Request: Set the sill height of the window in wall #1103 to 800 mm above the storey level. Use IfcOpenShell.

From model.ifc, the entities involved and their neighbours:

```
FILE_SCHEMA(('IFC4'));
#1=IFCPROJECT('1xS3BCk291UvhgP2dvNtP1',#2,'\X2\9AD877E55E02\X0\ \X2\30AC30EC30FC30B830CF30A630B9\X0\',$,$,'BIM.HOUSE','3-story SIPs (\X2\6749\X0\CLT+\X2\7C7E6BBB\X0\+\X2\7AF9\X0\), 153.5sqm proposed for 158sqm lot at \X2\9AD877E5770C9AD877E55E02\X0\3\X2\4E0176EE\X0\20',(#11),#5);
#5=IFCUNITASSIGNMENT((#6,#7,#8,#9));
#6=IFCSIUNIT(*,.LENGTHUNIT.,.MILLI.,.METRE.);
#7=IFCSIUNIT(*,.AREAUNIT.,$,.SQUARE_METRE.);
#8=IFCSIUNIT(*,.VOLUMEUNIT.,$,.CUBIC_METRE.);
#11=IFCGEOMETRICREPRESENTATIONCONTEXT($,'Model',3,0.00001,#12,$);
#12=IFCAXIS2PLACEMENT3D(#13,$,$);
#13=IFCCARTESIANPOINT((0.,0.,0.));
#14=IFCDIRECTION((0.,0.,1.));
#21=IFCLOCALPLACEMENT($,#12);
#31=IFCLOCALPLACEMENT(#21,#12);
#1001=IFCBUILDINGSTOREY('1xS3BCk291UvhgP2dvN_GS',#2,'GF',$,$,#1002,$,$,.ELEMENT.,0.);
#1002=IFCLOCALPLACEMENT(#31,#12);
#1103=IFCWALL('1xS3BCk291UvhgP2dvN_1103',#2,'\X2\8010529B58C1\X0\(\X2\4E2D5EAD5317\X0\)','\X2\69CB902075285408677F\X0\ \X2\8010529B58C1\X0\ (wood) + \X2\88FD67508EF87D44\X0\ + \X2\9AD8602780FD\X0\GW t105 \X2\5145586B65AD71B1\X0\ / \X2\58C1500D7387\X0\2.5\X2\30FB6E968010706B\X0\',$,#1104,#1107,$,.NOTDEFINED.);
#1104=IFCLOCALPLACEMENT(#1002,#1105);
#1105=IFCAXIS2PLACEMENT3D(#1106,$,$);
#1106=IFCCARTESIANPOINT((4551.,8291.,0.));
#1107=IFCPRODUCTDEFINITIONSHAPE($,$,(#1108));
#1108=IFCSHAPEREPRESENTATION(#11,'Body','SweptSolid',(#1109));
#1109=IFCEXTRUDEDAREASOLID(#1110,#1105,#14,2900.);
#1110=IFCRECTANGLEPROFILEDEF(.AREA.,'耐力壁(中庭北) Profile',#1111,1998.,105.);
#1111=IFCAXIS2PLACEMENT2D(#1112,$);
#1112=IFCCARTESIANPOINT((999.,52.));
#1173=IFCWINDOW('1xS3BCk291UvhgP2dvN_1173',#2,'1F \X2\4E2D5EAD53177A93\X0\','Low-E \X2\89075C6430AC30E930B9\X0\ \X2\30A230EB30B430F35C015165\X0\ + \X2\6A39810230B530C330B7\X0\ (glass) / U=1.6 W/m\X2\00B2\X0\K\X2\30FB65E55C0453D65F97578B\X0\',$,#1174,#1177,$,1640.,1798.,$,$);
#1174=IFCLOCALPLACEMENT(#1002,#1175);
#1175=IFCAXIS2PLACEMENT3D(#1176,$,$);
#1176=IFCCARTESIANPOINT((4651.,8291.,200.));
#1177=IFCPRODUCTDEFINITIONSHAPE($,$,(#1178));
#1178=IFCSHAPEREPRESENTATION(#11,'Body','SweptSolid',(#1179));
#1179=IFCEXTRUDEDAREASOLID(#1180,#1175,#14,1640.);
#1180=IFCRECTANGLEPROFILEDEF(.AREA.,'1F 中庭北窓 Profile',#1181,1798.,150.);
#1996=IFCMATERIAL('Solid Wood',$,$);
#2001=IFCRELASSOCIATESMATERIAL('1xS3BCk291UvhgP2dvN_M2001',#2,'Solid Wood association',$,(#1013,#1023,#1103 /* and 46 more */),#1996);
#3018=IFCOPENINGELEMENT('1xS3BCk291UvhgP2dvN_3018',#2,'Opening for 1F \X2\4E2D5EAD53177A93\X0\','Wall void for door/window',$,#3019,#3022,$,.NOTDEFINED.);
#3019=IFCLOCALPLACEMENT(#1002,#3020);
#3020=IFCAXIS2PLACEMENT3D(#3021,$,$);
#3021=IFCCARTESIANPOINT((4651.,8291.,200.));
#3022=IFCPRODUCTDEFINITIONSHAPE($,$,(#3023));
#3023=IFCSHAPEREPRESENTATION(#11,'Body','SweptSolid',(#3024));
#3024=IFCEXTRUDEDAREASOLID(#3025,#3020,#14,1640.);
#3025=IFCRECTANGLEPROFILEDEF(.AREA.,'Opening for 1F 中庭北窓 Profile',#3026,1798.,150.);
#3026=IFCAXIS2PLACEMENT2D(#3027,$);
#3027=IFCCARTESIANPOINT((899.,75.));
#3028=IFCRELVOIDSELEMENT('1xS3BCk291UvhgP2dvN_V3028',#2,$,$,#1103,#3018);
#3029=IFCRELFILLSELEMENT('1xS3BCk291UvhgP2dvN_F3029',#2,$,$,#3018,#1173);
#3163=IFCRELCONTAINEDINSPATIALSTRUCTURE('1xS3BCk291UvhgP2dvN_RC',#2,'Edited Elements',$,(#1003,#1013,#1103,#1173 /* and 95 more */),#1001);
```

```python
import numpy as np
import ifcopenshell
import ifcopenshell.api.geometry
import ifcopenshell.geom
import ifcopenshell.util.element
import ifcopenshell.util.placement
import ifcopenshell.util.shape
import ifcopenshell.util.unit

model = ifcopenshell.open("model.ifc")
unit_scale = ifcopenshell.util.unit.calculate_unit_scale(model)

window = model.by_guid("1xS3BCk291UvhgP2dvN_1173")
opening = window.FillsVoids[0].RelatingOpeningElement
storey = ifcopenshell.util.element.get_container(window, ifc_class="IfcBuildingStorey")
level = ifcopenshell.util.placement.get_local_placement(storey.ObjectPlacement)[2, 3]

# The opening's origin need not be at the sill, so measure its lowest point.
shape = ifcopenshell.geom.create_shape(ifcopenshell.geom.settings(), opening)
bottom = ifcopenshell.util.shape.get_shape_bottom_elevation(shape, shape.geometry) / unit_scale
dz = level + 0.8 / unit_scale - bottom

shift = np.array([0.0, 0.0, dz])
# The window is not placed relative to its opening, so move both.
for product in (opening, window):
    matrix = ifcopenshell.util.placement.get_local_placement(product.ObjectPlacement)
    matrix[:3, 3] += shift
    ifcopenshell.api.geometry.edit_object_placement(model, product=product, matrix=matrix, is_si=False)

print(f"moved by {dz * unit_scale:+.3f} m")

model.write("model_v2.ifc")
```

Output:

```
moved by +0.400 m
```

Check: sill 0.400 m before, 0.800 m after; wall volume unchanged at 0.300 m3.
